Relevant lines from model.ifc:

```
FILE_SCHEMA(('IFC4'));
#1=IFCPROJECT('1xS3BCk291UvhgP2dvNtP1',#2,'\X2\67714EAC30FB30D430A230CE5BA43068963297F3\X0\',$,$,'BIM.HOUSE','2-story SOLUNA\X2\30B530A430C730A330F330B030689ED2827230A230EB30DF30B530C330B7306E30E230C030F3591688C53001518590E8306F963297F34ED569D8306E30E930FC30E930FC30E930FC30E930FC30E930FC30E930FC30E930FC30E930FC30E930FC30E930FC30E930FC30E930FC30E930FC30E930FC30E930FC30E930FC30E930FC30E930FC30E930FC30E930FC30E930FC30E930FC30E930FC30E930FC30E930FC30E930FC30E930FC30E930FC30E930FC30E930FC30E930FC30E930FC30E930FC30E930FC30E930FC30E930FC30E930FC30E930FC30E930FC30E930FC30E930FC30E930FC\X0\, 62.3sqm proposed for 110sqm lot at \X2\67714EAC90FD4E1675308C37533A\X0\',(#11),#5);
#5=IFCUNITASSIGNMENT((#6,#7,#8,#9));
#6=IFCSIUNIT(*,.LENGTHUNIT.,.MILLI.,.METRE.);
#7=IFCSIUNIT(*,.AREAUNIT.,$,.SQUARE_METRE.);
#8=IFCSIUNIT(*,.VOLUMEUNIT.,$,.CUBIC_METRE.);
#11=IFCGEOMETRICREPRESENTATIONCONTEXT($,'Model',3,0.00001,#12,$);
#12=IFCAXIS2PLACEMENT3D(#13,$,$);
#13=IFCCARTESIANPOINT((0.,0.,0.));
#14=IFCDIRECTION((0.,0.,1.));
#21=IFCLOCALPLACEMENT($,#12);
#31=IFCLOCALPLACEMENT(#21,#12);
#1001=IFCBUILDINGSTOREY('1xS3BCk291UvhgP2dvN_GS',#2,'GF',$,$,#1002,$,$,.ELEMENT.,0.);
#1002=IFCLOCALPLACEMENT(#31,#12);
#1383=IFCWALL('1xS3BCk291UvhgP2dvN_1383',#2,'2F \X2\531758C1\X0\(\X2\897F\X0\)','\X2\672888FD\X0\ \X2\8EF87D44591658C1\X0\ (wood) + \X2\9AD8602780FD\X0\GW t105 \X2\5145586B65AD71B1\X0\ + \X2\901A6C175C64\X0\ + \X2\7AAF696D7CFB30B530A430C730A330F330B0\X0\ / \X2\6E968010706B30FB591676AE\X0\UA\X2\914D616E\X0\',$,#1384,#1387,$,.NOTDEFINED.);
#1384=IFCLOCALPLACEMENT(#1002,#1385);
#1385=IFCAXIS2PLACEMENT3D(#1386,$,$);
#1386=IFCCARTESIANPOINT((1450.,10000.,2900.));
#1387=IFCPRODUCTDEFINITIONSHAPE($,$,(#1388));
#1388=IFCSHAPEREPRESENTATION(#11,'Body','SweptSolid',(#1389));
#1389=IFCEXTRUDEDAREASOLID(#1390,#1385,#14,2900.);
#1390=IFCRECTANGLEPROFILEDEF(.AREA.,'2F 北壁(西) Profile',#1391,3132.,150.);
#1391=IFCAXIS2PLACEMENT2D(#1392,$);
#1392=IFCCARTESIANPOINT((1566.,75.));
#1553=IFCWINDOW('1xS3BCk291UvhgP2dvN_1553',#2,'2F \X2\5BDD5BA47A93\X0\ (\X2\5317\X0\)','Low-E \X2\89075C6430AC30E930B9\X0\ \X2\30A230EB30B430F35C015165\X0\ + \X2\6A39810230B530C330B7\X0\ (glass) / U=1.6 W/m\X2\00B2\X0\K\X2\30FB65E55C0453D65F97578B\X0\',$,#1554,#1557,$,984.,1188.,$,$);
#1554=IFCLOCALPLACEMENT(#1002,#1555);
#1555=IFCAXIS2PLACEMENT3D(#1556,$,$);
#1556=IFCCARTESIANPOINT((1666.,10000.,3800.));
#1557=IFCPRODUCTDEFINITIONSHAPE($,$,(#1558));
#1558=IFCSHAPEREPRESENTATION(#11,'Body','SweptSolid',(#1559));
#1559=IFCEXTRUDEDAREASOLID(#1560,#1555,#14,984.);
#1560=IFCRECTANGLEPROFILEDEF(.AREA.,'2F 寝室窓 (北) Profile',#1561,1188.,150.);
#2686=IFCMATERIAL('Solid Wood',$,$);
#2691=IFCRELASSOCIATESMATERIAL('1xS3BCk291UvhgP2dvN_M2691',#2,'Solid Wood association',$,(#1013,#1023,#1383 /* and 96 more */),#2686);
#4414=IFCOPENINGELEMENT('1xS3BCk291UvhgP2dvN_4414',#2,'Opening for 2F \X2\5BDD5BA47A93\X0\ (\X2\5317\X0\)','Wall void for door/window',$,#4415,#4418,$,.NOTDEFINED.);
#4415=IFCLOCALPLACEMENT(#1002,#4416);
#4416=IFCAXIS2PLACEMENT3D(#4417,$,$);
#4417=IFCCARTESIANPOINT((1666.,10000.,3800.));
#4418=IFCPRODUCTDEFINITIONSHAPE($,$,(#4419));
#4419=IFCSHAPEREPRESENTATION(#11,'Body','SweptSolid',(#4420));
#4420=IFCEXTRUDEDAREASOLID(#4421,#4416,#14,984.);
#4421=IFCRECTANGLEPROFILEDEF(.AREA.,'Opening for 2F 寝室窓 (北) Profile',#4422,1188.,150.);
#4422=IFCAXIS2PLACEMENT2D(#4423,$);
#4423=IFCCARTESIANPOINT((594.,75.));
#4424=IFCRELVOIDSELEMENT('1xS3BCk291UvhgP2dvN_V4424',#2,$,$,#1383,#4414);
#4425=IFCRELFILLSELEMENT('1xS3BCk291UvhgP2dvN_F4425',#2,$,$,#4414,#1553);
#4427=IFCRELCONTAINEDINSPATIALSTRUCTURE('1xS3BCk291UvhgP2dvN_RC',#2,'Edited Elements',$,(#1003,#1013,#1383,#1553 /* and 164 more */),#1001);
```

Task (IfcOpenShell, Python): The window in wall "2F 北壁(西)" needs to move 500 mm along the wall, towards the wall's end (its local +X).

```python
import ifcopenshell
import ifcopenshell.api.geometry
import ifcopenshell.util.placement
import ifcopenshell.util.unit

model = ifcopenshell.open("model.ifc")
unit_scale = ifcopenshell.util.unit.calculate_unit_scale(model)

window = model.by_id(1553)
opening = window.FillsVoids[0].RelatingOpeningElement
wall = opening.VoidsElements[0].RelatingBuildingElement

wall_matrix = ifcopenshell.util.placement.get_local_placement(wall.ObjectPlacement)
shift = wall_matrix[:3, 0] * 0.5 / unit_scale
before = ifcopenshell.util.placement.get_local_placement(window.ObjectPlacement)[:3, 3].copy()

# The window is not placed relative to its opening, so move both.
for product in (opening, window):
    matrix = ifcopenshell.util.placement.get_local_placement(product.ObjectPlacement)
    matrix[:3, 3] += shift
    ifcopenshell.api.geometry.edit_object_placement(model, product=product, matrix=matrix, is_si=False)

after = ifcopenshell.util.placement.get_local_placement(window.ObjectPlacement)[:3, 3]
print("window moved by", (after - before).round(3) + 0.0)

model.write("model-out.ifc")
```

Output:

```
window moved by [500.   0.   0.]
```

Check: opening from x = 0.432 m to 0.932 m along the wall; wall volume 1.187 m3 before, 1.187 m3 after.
